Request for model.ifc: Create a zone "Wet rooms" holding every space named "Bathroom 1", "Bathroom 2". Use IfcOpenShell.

First a look at what the model holds.

```python
import ifcopenshell

model = ifcopenshell.open("model.ifc")
print(model.schema)
seen = {}
for space in model.by_type("IfcSpace"):
    seen[space.LongName] = seen.get(space.LongName, 0) + 1
for name, count in sorted(seen.items(), key=str):
    print(count, "x", name)
print("zones:", [z.Name for z in model.by_type("IfcZone")][:20])
```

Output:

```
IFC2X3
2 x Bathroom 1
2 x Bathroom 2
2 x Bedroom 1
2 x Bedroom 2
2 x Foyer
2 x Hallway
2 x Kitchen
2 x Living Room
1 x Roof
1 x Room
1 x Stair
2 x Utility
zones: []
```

```python
import ifcopenshell
import ifcopenshell.api.group
import ifcopenshell.api.root

model = ifcopenshell.open("model.ifc")

names = {"Bathroom 1", "Bathroom 2"}
spaces = [s for s in model.by_type("IfcSpace") if s.LongName in names]

zone = ifcopenshell.api.root.create_entity(model, ifc_class="IfcZone", name="Wet rooms")
ifcopenshell.api.group.assign_group(model, products=spaces, group=zone)
print(len(spaces), "spaces in", zone.Name)

model.write("model-out.ifc")
```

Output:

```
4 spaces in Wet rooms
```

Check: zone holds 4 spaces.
